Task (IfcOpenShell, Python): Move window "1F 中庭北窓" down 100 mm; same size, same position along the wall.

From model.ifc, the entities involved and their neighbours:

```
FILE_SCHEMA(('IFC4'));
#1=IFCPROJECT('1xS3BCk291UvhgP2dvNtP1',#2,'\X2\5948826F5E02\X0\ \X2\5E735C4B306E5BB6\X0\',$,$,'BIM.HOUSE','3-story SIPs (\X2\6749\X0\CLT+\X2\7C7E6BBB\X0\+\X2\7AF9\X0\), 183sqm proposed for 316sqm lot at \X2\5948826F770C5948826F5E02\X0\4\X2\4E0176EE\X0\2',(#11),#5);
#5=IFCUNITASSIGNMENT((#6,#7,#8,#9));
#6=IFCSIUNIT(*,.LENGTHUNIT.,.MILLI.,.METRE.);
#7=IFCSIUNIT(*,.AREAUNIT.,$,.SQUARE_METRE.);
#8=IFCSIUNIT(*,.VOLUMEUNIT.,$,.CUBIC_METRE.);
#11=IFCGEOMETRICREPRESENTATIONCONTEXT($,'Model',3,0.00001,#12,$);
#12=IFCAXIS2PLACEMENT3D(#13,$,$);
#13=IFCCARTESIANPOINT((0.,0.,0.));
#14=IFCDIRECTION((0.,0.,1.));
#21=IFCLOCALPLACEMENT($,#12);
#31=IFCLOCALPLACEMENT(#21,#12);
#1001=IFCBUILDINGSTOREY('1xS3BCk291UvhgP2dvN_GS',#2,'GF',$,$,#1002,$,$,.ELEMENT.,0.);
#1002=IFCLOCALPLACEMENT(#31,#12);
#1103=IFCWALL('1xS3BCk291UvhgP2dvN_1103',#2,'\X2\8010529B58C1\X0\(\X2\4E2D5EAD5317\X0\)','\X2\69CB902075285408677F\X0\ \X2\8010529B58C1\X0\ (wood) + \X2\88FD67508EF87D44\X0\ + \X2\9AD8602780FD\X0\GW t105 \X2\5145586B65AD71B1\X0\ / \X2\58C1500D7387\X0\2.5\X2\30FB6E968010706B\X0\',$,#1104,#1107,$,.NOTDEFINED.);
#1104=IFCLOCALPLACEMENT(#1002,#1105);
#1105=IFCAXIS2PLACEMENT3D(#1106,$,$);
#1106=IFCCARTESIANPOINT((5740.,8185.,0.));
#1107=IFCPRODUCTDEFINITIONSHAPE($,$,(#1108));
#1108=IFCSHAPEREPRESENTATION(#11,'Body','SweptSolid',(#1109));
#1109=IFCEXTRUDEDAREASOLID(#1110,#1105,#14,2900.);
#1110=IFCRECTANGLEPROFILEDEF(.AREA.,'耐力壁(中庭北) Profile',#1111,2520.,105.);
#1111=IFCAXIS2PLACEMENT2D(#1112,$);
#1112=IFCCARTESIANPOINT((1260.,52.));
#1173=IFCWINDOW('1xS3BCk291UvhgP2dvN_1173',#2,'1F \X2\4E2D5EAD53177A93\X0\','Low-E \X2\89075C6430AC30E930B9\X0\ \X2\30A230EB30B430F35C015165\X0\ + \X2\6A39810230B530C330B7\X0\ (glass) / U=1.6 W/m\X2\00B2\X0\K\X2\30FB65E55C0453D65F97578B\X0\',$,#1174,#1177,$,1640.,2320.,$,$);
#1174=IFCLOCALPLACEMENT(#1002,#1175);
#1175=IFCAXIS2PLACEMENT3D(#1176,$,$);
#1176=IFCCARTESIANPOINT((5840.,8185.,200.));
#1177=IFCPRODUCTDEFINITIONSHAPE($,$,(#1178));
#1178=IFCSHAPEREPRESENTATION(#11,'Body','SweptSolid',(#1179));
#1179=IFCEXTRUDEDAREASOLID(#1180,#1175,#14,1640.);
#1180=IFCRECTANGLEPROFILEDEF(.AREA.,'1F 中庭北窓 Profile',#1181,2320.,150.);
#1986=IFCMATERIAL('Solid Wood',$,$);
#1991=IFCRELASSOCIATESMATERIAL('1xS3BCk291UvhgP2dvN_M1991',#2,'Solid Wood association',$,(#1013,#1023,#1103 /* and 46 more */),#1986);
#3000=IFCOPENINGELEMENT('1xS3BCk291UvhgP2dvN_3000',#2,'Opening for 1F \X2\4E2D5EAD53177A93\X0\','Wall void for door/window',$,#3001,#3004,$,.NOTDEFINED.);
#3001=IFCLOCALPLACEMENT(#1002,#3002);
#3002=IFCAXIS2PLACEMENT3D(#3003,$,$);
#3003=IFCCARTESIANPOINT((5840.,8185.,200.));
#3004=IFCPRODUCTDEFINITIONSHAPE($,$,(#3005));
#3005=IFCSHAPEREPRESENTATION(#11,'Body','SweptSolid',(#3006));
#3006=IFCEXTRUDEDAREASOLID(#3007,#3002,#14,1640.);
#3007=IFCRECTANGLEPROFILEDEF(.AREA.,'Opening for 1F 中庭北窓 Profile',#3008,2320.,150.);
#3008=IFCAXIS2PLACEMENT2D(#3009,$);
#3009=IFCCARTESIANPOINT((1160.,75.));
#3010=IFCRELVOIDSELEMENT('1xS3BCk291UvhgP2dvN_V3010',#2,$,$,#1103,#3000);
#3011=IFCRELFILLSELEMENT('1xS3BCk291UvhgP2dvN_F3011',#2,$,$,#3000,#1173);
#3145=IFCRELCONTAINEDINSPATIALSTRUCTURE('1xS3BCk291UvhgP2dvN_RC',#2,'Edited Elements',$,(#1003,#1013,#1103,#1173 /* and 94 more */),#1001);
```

```python
import numpy as np
import ifcopenshell
import ifcopenshell.api.geometry
import ifcopenshell.util.placement
import ifcopenshell.util.unit

model = ifcopenshell.open("model.ifc")
unit_scale = ifcopenshell.util.unit.calculate_unit_scale(model)

window = model.by_guid("1xS3BCk291UvhgP2dvN_1173")
opening = window.FillsVoids[0].RelatingOpeningElement
dz = -0.1 / unit_scale

shift = np.array([0.0, 0.0, dz])
# The window is not placed relative to its opening, so move both.
for product in (opening, window):
    matrix = ifcopenshell.util.placement.get_local_placement(product.ObjectPlacement)
    matrix[:3, 3] += shift
    ifcopenshell.api.geometry.edit_object_placement(model, product=product, matrix=matrix, is_si=False)

print(f"moved by {dz * unit_scale:+.3f} m")

model.write("model_v2.ifc")
```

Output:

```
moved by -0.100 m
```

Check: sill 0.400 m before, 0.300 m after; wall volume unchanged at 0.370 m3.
